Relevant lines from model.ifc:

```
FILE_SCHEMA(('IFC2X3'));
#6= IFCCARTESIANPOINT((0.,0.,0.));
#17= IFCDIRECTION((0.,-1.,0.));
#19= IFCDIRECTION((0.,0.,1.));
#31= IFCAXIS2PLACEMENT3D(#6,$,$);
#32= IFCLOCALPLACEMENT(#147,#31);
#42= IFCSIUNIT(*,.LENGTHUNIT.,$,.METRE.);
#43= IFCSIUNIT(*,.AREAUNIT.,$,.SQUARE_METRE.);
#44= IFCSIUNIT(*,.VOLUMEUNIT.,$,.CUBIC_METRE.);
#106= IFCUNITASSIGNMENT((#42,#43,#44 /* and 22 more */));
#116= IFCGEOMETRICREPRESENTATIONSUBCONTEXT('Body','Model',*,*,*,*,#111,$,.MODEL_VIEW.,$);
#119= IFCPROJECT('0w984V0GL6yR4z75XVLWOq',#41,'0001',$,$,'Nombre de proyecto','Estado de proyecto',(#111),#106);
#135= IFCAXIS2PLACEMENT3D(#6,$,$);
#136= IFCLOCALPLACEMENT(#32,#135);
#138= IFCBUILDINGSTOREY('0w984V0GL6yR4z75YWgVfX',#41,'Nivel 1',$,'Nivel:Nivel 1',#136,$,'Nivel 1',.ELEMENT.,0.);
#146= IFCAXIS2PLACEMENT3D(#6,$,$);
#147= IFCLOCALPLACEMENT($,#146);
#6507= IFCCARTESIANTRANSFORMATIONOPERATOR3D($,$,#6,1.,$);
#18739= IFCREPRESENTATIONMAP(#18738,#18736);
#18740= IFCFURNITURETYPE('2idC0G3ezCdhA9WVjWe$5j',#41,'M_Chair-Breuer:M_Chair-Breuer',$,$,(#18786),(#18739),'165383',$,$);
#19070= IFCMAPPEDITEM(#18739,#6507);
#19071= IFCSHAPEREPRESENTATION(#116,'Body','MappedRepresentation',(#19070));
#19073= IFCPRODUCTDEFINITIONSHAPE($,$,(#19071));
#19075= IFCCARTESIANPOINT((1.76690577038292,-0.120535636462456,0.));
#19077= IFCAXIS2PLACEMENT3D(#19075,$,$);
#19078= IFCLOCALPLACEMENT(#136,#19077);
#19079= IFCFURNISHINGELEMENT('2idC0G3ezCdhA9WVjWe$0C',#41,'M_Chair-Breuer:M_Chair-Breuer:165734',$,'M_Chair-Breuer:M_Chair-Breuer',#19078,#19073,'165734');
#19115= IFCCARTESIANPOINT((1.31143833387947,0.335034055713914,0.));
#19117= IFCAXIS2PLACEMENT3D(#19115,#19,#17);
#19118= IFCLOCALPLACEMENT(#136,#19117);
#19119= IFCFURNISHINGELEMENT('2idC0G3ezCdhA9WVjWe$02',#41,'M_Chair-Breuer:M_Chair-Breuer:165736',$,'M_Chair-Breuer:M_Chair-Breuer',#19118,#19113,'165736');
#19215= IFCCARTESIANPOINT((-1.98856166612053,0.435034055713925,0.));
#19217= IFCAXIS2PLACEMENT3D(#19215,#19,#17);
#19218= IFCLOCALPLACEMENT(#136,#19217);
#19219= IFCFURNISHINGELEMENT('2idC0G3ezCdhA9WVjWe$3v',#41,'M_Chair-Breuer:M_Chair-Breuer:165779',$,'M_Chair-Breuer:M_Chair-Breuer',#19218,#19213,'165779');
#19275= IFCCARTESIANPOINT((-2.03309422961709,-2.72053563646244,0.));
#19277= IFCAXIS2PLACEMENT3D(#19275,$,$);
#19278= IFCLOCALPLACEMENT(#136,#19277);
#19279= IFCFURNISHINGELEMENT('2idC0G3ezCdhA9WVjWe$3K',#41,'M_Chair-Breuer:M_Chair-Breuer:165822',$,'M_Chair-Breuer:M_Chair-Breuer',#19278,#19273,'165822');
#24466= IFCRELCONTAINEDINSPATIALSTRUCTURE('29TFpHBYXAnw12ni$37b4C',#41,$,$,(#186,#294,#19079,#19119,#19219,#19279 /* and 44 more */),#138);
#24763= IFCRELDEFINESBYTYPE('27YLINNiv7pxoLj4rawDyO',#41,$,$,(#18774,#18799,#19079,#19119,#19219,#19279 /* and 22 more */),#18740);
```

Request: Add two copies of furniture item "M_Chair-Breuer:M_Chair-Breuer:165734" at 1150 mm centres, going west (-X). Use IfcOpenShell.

```python
import numpy as np
import ifcopenshell
import ifcopenshell.api.geometry
import ifcopenshell.api.root
import ifcopenshell.util.element
import ifcopenshell.util.placement
import ifcopenshell.util.unit

model = ifcopenshell.open("model.ifc")
unit_scale = ifcopenshell.util.unit.calculate_unit_scale(model)


def reuse_history(source, copy):
    """copy_class also copies each property set's owner history, people and application; keep the originals."""
    for rel in copy.IsDefinedBy:
        if rel.is_a("IfcRelDefinesByProperties") and (history := rel.RelatingPropertyDefinition.OwnerHistory):
            rel.RelatingPropertyDefinition.OwnerHistory = source.OwnerHistory
            ifcopenshell.util.element.remove_deep2(model, history)


source = model.by_guid("2idC0G3ezCdhA9WVjWe$0C")
base = ifcopenshell.util.placement.get_local_placement(source.ObjectPlacement)
step = np.array([-1.0, 0.0, 0.0]) * 1.15 / unit_scale

for i in range(1, 3):
    copy = ifcopenshell.api.root.copy_class(model, product=source)
    copy.Representation = ifcopenshell.util.element.copy_deep(
        model, source.Representation, exclude=["IfcGeometricRepresentationContext", "IfcRepresentationMap"]
    )
    copy.Name = "M_Chair-Breuer:M_Chair-Breuer"
    copy.Tag = None
    reuse_history(source, copy)
    matrix = base.copy()
    matrix[:3, 3] += i * step
    print("added at", matrix[:3, 3].round(3) + 0.0)
    ifcopenshell.api.geometry.edit_object_placement(model, product=copy, matrix=matrix, is_si=False)

model.write("model_v2.ifc")
```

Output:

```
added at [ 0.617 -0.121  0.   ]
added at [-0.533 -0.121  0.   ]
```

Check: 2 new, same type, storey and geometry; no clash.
